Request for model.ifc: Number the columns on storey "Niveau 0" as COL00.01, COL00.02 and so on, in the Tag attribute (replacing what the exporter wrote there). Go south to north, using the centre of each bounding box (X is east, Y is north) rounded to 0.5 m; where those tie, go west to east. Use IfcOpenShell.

First a look at what the model holds.

```python
import ifcopenshell
import ifcopenshell.util.element
import ifcopenshell.util.placement

model = ifcopenshell.open("model.ifc")
print(model.schema)
storey = next(s for s in model.by_type("IfcBuildingStorey") if s.Name == "Niveau 0")
columns = [e for e in ifcopenshell.util.element.get_decomposition(storey) if e.is_a("IfcColumn")]
for e in sorted(columns, key=lambda e: e.id()):
    origin = ifcopenshell.util.placement.get_local_placement(e.ObjectPlacement)[:3, 3]
    print(e.id(), e.Tag, e.Name, origin.round(2) + 0.0, sep=" | ")
```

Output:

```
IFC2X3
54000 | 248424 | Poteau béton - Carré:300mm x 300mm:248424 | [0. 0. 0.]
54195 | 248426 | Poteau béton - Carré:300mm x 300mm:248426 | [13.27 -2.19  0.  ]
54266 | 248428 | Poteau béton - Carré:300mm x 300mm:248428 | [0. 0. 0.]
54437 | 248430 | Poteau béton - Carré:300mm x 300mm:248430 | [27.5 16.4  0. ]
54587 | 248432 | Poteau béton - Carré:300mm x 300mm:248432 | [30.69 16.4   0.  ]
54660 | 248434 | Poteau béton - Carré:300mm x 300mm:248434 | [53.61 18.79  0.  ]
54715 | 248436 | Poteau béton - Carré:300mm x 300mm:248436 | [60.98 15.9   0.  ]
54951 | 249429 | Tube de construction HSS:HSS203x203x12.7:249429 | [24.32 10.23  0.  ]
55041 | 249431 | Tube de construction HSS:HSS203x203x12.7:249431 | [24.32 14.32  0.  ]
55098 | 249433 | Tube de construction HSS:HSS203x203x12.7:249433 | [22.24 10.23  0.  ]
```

```python
import ifcopenshell
import ifcopenshell.geom
import ifcopenshell.util.element
import ifcopenshell.util.shape

model = ifcopenshell.open("model.ifc")
settings = ifcopenshell.geom.settings()
settings.set("use-world-coords", True)


def centre(element):
    shape = ifcopenshell.geom.create_shape(settings, element)
    return ifcopenshell.util.shape.get_bbox_centroid(shape.geometry)


storey = next(s for s in model.by_type("IfcBuildingStorey") if s.Name == "Niveau 0")
columns = [e for e in ifcopenshell.util.element.get_decomposition(storey) if e.is_a("IfcColumn")]

# Insertion points can sit at a corner or the storey origin, so sort by the geometry (in metres).
centres = {e: centre(e) for e in columns}
columns.sort(key=lambda e: (round(centres[e][1] / 0.5), centres[e][0]))

for i, e in enumerate(columns, start=1):
    number = f"COL00.{i:02d}"
    e.Tag = number
    print(e.id(), number)

model.write("model_edited.ifc")
```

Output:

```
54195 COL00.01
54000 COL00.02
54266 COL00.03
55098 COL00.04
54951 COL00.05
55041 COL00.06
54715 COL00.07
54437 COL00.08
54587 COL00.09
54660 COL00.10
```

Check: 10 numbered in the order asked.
